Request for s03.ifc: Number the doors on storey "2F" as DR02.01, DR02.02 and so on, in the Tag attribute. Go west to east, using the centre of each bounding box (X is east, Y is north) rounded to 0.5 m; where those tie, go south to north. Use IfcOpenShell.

First a look at what the model holds.

```python
import ifcopenshell
import ifcopenshell.util.element
import ifcopenshell.util.placement

model = ifcopenshell.open("s03.ifc")
print(model.schema)
storey = next(s for s in model.by_type("IfcBuildingStorey") if s.Name == "2F")
doors = [e for e in ifcopenshell.util.element.get_decomposition(storey) if e.is_a("IfcDoor")]
for e in sorted(doors, key=lambda e: e.id()):
    origin = ifcopenshell.util.placement.get_local_placement(e.ObjectPlacement)[:3, 3]
    print(e.id(), e.Tag, e.Name, origin.round(2) + 0.0, sep=" | ")
```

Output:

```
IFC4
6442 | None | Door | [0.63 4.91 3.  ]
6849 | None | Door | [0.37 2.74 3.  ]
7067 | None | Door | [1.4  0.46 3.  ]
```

```python
import ifcopenshell
import ifcopenshell.geom
import ifcopenshell.util.element
import ifcopenshell.util.shape

model = ifcopenshell.open("s03.ifc")
settings = ifcopenshell.geom.settings()
settings.set("use-world-coords", True)


def centre(element):
    shape = ifcopenshell.geom.create_shape(settings, element)
    return ifcopenshell.util.shape.get_bbox_centroid(shape.geometry)


storey = next(s for s in model.by_type("IfcBuildingStorey") if s.Name == "2F")
doors = [e for e in ifcopenshell.util.element.get_decomposition(storey) if e.is_a("IfcDoor")]

# Insertion points can sit at a corner or the storey origin, so sort by the geometry (in metres).
centres = {e: centre(e) for e in doors}
doors.sort(key=lambda e: (round(centres[e][0] / 0.5), centres[e][1]))

for i, e in enumerate(doors, start=1):
    number = f"DR02.{i:02d}"
    e.Tag = number
    print(e.id(), number)

model.write("s03_updated.ifc")
```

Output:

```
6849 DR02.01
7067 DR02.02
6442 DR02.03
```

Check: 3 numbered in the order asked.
